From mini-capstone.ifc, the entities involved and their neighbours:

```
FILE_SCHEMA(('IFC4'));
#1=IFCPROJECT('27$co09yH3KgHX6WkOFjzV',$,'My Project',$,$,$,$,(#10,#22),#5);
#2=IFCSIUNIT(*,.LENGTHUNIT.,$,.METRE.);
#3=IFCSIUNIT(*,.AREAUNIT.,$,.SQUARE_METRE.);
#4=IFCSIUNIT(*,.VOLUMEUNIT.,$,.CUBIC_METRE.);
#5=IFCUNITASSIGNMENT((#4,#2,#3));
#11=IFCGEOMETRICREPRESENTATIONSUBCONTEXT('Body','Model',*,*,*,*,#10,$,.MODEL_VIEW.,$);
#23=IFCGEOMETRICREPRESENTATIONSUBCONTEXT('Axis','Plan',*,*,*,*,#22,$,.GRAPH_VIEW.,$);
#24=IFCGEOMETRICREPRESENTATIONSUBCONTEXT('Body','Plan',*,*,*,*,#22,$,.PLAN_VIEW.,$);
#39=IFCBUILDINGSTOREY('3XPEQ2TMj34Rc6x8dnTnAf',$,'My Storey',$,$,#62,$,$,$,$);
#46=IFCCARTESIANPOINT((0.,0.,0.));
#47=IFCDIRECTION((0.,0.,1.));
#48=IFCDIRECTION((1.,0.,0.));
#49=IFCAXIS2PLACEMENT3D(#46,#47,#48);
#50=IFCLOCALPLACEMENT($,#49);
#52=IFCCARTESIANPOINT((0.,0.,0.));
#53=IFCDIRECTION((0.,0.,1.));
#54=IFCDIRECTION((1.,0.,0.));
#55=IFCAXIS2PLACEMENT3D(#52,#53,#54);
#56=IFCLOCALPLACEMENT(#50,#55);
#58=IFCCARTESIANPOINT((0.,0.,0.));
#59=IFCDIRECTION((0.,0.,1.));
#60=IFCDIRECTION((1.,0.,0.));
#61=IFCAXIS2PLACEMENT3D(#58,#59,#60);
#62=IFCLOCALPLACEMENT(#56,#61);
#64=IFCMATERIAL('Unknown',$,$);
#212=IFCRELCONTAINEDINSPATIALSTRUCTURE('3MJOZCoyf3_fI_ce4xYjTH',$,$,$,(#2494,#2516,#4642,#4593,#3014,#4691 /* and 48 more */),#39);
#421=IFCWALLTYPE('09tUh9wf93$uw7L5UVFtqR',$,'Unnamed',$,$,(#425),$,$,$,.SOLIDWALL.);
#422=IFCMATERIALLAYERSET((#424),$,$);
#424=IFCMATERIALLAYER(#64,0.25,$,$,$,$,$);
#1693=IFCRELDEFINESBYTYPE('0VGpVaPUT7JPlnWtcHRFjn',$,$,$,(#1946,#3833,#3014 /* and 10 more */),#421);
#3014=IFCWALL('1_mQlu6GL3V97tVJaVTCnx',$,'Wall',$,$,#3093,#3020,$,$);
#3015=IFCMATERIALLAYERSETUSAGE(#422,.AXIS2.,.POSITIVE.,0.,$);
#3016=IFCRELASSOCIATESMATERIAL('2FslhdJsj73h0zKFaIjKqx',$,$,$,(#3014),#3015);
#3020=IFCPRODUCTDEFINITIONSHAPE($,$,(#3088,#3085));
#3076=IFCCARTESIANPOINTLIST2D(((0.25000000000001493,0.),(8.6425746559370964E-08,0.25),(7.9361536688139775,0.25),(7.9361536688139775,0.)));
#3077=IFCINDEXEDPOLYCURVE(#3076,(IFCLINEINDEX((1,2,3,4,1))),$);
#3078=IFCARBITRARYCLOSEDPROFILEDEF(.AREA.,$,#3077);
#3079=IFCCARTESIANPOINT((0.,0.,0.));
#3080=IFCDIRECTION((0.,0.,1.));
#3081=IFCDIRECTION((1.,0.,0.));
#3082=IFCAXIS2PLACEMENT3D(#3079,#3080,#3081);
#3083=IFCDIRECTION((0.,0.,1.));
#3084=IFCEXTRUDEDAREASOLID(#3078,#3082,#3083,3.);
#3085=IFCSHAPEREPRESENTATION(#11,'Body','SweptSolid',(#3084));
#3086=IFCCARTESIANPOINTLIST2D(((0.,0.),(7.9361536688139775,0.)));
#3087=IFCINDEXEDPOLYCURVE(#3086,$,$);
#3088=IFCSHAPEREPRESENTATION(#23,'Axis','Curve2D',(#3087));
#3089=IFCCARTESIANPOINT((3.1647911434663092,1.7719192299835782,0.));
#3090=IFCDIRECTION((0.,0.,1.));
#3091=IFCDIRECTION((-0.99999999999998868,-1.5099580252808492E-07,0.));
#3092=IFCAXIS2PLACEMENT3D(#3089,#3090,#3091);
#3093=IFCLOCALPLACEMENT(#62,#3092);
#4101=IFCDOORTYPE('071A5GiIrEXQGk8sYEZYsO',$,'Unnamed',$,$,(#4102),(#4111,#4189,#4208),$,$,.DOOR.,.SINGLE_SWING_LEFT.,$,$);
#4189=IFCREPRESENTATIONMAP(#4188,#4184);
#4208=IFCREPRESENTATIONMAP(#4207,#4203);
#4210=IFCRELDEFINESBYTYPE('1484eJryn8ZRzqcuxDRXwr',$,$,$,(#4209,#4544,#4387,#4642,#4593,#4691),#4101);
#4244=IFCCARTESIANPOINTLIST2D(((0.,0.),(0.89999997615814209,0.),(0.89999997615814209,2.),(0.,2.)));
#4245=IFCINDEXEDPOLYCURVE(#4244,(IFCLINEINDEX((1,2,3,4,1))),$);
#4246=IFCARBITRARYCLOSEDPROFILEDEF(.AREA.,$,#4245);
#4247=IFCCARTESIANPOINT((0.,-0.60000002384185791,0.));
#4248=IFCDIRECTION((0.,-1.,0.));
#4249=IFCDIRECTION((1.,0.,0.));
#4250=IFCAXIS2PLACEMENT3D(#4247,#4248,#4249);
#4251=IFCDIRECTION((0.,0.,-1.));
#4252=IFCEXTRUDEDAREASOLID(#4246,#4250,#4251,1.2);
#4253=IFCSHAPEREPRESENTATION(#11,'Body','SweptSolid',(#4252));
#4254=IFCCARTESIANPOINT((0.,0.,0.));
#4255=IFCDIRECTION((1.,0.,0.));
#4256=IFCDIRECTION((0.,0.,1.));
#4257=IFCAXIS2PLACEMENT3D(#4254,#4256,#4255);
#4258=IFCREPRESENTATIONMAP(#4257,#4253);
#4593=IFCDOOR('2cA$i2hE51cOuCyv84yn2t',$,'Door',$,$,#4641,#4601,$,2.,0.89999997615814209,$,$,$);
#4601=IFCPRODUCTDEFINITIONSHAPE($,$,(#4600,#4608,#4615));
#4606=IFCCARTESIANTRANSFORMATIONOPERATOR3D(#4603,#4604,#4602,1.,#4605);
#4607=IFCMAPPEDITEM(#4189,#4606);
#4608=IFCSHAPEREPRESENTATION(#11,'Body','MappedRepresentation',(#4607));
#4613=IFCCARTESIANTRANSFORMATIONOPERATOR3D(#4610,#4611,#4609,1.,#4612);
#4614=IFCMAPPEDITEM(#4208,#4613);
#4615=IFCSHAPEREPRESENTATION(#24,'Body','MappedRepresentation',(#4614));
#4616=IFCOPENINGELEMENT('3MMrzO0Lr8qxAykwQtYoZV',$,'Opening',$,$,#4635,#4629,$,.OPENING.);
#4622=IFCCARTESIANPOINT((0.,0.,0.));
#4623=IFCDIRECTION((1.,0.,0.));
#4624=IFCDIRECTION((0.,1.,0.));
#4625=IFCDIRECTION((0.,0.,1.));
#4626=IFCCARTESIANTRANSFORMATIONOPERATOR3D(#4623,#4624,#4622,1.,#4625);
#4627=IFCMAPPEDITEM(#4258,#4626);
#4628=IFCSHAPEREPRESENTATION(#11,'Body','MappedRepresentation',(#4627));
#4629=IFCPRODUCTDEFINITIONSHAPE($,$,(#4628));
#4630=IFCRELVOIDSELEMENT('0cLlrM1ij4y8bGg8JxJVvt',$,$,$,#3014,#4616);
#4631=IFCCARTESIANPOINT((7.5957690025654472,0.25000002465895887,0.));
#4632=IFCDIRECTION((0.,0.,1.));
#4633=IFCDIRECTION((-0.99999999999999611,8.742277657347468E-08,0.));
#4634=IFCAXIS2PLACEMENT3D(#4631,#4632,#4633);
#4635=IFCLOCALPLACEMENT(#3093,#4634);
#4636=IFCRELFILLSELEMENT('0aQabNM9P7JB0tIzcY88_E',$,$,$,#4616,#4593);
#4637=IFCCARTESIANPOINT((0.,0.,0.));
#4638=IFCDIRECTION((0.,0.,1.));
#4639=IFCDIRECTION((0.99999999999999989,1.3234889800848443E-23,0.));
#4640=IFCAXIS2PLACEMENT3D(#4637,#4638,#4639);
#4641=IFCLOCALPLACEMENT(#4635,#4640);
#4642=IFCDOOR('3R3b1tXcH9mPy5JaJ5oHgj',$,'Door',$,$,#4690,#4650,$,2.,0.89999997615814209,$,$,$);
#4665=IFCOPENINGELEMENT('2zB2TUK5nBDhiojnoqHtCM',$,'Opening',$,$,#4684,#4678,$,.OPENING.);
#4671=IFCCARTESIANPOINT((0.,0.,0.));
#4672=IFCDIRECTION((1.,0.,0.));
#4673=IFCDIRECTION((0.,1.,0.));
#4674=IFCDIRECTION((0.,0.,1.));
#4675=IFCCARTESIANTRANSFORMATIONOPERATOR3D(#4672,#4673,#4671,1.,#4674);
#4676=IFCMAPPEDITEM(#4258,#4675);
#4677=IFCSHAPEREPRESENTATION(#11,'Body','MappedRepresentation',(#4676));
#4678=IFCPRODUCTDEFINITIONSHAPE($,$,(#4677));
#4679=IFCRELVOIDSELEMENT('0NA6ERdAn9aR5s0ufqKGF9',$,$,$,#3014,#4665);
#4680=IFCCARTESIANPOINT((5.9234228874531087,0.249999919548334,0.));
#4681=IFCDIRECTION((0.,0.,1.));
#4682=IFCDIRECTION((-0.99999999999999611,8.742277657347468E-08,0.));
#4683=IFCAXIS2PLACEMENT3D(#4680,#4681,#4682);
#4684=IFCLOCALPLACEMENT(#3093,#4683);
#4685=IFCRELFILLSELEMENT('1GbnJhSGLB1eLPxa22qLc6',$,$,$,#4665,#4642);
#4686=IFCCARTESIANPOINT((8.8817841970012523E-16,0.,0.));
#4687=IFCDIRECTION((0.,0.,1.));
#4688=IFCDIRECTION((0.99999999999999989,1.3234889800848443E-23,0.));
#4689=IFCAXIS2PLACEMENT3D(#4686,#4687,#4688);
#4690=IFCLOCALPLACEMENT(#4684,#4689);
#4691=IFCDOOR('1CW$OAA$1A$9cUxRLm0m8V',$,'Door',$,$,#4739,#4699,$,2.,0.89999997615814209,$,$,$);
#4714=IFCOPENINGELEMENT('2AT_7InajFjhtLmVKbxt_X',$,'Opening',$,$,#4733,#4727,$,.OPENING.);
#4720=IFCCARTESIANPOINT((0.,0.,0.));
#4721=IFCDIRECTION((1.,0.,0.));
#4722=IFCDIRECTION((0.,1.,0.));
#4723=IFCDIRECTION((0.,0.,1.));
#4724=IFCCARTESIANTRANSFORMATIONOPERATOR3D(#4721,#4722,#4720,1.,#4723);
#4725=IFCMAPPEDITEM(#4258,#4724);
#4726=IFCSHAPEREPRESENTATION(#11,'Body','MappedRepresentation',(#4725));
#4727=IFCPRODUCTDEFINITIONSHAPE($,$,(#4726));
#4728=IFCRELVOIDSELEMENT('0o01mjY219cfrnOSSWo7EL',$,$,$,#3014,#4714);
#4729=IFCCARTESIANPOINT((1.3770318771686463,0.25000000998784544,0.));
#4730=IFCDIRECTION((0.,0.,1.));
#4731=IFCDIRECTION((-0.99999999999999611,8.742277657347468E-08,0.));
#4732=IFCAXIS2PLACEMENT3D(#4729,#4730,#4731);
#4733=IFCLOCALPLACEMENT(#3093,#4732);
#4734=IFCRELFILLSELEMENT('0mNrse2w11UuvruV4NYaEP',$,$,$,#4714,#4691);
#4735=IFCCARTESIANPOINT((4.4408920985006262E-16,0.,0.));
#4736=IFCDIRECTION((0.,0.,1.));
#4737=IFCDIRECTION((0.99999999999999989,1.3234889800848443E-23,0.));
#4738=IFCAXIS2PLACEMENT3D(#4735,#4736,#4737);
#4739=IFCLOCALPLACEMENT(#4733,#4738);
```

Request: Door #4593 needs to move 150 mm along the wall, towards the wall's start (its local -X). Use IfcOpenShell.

```python
import ifcopenshell
import ifcopenshell.api.geometry
import ifcopenshell.util.placement
import ifcopenshell.util.unit

model = ifcopenshell.open("mini-capstone.ifc")
unit_scale = ifcopenshell.util.unit.calculate_unit_scale(model)

door = model.by_guid("2cA$i2hE51cOuCyv84yn2t")
opening = door.FillsVoids[0].RelatingOpeningElement
wall = opening.VoidsElements[0].RelatingBuildingElement

wall_matrix = ifcopenshell.util.placement.get_local_placement(wall.ObjectPlacement)
shift = wall_matrix[:3, 0] * -0.15 / unit_scale
before = ifcopenshell.util.placement.get_local_placement(door.ObjectPlacement)[:3, 3].copy()

# The door is placed relative to its opening, so it follows when the opening moves.
matrix = ifcopenshell.util.placement.get_local_placement(opening.ObjectPlacement)
matrix[:3, 3] += shift
ifcopenshell.api.geometry.edit_object_placement(
    model, product=opening, matrix=matrix, is_si=False, should_transform_children=True
)

after = ifcopenshell.util.placement.get_local_placement(door.ObjectPlacement)[:3, 3]
print("door moved by", (after - before).round(3) + 0.0)

model.write("mini-capstone_edited.ifc")
```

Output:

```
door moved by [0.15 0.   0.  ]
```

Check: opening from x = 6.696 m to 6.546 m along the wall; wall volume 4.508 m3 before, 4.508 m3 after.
